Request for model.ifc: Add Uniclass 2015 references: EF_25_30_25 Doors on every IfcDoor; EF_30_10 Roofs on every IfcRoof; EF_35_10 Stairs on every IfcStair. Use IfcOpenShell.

First a look at what the model holds.

```python
import ifcopenshell

model = ifcopenshell.open("model.ifc")
print(model.schema)
print("classifications:", [c.Name for c in model.by_type("IfcClassification")])
for ifc_class in ("IfcDoor", "IfcRoof", "IfcStair", "IfcWall", "IfcWindow"):
    print(ifc_class, len(model.by_type(ifc_class)))
```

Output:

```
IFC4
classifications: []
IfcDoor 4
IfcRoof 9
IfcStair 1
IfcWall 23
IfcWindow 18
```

```python
import ifcopenshell
import ifcopenshell.api.classification

model = ifcopenshell.open("model.ifc")

system = ifcopenshell.api.classification.add_classification(model, classification="Uniclass 2015")

codes = {
    "IfcDoor": ("EF_25_30_25", "Doors"),
    "IfcRoof": ("EF_30_10", "Roofs"),
    "IfcStair": ("EF_35_10", "Stairs"),
}
for ifc_class, (code, name) in codes.items():
    products = model.by_type(ifc_class)
    ifcopenshell.api.classification.add_reference(
        model, products=products, classification=system, identification=code, name=name
    )
    print(code, len(products))

model.write("model_rev.ifc")
```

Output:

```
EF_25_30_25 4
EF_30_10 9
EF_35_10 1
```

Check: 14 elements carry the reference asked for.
